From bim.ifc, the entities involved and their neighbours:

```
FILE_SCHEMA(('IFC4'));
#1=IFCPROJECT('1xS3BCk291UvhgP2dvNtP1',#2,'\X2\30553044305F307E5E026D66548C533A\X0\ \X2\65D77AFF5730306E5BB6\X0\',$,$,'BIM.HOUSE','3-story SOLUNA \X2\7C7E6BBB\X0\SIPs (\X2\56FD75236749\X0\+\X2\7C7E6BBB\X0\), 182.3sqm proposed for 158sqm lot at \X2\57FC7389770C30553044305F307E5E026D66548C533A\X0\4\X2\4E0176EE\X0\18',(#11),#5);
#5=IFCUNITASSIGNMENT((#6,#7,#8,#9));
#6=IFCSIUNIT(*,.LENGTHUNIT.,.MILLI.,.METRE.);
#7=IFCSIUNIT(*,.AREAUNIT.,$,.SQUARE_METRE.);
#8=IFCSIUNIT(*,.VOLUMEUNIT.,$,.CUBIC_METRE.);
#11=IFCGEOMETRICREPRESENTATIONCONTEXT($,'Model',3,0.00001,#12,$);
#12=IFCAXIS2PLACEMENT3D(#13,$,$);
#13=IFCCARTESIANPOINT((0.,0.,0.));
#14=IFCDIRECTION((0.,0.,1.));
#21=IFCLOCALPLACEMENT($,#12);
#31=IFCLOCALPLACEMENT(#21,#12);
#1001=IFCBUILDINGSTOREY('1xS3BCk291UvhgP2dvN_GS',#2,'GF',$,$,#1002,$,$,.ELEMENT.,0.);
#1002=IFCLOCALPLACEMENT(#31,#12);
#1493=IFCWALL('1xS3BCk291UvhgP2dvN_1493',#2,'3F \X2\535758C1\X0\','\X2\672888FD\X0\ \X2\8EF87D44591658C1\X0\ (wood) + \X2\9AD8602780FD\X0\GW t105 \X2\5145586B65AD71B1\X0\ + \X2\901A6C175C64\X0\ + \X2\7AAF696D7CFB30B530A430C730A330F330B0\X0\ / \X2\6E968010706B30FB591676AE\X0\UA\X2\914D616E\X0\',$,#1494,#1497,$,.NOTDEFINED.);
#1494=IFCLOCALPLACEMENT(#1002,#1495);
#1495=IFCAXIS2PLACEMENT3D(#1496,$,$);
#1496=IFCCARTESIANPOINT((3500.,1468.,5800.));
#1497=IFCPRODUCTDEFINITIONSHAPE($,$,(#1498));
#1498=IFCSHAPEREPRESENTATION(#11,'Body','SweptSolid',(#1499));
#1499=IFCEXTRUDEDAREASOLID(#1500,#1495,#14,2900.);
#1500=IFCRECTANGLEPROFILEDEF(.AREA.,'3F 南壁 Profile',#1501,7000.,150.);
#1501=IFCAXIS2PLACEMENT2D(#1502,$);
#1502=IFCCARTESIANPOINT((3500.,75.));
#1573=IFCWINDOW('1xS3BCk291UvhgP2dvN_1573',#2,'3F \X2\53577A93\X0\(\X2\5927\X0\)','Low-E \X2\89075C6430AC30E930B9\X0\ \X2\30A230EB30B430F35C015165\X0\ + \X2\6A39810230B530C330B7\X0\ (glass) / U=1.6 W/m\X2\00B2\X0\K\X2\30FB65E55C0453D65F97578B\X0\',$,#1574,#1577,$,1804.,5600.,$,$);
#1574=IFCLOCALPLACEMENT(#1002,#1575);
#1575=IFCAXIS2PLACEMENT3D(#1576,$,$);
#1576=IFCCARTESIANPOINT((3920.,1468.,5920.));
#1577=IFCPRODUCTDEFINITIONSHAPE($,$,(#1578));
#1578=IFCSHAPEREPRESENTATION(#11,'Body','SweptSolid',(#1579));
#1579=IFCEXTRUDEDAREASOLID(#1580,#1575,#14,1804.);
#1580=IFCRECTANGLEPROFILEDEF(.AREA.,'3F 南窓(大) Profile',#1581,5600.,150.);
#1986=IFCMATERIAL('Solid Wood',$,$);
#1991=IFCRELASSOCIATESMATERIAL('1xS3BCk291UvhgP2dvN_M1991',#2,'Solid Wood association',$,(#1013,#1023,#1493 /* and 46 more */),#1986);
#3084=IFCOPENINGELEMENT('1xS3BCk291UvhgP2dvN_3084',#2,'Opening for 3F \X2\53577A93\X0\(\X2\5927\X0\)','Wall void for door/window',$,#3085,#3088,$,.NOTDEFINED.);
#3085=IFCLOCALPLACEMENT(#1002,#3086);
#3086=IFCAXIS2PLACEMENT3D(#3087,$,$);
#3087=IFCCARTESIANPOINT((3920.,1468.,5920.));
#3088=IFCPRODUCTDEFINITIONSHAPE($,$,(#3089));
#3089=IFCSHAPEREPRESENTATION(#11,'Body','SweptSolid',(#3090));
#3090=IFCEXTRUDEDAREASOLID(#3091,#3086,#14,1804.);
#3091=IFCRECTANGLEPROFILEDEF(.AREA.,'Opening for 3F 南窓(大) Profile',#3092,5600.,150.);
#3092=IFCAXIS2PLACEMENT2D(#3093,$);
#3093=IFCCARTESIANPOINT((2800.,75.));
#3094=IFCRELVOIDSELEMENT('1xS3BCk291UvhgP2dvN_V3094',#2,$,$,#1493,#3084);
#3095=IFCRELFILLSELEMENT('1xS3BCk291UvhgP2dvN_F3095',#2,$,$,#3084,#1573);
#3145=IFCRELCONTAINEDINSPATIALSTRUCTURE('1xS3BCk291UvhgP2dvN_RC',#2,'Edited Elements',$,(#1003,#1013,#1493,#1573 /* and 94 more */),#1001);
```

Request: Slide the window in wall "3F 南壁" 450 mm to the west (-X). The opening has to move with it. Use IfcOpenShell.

```python
import ifcopenshell
import ifcopenshell.api.geometry
import ifcopenshell.util.placement
import ifcopenshell.util.unit

model = ifcopenshell.open("bim.ifc")
unit_scale = ifcopenshell.util.unit.calculate_unit_scale(model)

window = model.by_guid("1xS3BCk291UvhgP2dvN_1573")
opening = window.FillsVoids[0].RelatingOpeningElement
wall = opening.VoidsElements[0].RelatingBuildingElement

wall_matrix = ifcopenshell.util.placement.get_local_placement(wall.ObjectPlacement)
shift = wall_matrix[:3, 0] * -0.45 / unit_scale
before = ifcopenshell.util.placement.get_local_placement(window.ObjectPlacement)[:3, 3].copy()

# The window is not placed relative to its opening, so move both.
for product in (opening, window):
    matrix = ifcopenshell.util.placement.get_local_placement(product.ObjectPlacement)
    matrix[:3, 3] += shift
    ifcopenshell.api.geometry.edit_object_placement(model, product=product, matrix=matrix, is_si=False)

after = ifcopenshell.util.placement.get_local_placement(window.ObjectPlacement)[:3, 3]
print("window moved by", (after - before).round(3) + 0.0)

model.write("bim_rev.ifc")
```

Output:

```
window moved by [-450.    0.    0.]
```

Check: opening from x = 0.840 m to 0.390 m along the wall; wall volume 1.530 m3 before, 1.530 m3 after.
